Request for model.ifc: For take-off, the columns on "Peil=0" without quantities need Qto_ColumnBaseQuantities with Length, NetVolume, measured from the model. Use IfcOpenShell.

First a look at what the model holds.

```python
import ifcopenshell
import ifcopenshell.util.element
import ifcopenshell.util.unit

model = ifcopenshell.open("model.ifc")
print(model.schema)
for unit_type in ("LENGTHUNIT", "AREAUNIT", "VOLUMEUNIT"):
    print(unit_type, ifcopenshell.util.unit.calculate_unit_scale(model, unit_type))
storey = next(s for s in model.by_type("IfcBuildingStorey") if s.Name == "Peil=0")
columns = [e for e in ifcopenshell.util.element.get_decomposition(storey) if e.is_a("IfcColumn")]
for e in sorted(columns, key=lambda e: e.id()):
    print(e.id(), e.is_a(), e.Name, list(ifcopenshell.util.element.get_psets(e, qtos_only=True)), sep=" | ")
```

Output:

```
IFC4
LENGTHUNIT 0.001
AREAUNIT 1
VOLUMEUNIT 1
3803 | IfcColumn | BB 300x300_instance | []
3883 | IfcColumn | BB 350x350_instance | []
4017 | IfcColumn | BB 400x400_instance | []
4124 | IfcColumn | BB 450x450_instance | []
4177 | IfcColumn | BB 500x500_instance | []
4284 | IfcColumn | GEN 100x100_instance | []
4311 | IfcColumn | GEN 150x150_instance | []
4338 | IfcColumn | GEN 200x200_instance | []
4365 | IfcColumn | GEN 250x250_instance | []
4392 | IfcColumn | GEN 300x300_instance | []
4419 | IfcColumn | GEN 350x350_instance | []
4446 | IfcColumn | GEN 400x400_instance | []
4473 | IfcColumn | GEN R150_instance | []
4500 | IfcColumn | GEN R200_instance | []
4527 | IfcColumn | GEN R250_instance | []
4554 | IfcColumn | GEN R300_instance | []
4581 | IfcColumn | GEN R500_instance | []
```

```python
import ifcopenshell
import ifcopenshell.api.pset
import ifcopenshell.geom
import ifcopenshell.util.element
import ifcopenshell.util.shape
import ifcopenshell.util.unit

model = ifcopenshell.open("model.ifc")
unit_scale = ifcopenshell.util.unit.calculate_unit_scale(model)
volume_scale = ifcopenshell.util.unit.calculate_unit_scale(model, "VOLUMEUNIT")
settings = ifcopenshell.geom.settings()

storey = next(s for s in model.by_type("IfcBuildingStorey") if s.Name == "Peil=0")
columns = [e for e in ifcopenshell.util.element.get_decomposition(storey) if e.is_a("IfcColumn")]

for e in sorted(columns, key=lambda e: e.id()):
    if ifcopenshell.util.element.get_psets(e, qtos_only=True, should_inherit=False):
        continue
    # Geometry comes back in metres, in the element's own axes.
    shape = ifcopenshell.geom.create_shape(settings, e)
    values = {
        "Length": ifcopenshell.util.shape.get_z(shape.geometry) / unit_scale,
        "NetVolume": ifcopenshell.util.shape.get_volume(shape.geometry) / volume_scale,
    }
    qto = ifcopenshell.api.pset.add_qto(model, product=e, name="Qto_ColumnBaseQuantities")
    ifcopenshell.api.pset.edit_qto(model, qto=qto, properties=values)
    print(e.id(), {k: round(v, 3) for k, v in values.items()})

model.write("model_updated.ifc")
```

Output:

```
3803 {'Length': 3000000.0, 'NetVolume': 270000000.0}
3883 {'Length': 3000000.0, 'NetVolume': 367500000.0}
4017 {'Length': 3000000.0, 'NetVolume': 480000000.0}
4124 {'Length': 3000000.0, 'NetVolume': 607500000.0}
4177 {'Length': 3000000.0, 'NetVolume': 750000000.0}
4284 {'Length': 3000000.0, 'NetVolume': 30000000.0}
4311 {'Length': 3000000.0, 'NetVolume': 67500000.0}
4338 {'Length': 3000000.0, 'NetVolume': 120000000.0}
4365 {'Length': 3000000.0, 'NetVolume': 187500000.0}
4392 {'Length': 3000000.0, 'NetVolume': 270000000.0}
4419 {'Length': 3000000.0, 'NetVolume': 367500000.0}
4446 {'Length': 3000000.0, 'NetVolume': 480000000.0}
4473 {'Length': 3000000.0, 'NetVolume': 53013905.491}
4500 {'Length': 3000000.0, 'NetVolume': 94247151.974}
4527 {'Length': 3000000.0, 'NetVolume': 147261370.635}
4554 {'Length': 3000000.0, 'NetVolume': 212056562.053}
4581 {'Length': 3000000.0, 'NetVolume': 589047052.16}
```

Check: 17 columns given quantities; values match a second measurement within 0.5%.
